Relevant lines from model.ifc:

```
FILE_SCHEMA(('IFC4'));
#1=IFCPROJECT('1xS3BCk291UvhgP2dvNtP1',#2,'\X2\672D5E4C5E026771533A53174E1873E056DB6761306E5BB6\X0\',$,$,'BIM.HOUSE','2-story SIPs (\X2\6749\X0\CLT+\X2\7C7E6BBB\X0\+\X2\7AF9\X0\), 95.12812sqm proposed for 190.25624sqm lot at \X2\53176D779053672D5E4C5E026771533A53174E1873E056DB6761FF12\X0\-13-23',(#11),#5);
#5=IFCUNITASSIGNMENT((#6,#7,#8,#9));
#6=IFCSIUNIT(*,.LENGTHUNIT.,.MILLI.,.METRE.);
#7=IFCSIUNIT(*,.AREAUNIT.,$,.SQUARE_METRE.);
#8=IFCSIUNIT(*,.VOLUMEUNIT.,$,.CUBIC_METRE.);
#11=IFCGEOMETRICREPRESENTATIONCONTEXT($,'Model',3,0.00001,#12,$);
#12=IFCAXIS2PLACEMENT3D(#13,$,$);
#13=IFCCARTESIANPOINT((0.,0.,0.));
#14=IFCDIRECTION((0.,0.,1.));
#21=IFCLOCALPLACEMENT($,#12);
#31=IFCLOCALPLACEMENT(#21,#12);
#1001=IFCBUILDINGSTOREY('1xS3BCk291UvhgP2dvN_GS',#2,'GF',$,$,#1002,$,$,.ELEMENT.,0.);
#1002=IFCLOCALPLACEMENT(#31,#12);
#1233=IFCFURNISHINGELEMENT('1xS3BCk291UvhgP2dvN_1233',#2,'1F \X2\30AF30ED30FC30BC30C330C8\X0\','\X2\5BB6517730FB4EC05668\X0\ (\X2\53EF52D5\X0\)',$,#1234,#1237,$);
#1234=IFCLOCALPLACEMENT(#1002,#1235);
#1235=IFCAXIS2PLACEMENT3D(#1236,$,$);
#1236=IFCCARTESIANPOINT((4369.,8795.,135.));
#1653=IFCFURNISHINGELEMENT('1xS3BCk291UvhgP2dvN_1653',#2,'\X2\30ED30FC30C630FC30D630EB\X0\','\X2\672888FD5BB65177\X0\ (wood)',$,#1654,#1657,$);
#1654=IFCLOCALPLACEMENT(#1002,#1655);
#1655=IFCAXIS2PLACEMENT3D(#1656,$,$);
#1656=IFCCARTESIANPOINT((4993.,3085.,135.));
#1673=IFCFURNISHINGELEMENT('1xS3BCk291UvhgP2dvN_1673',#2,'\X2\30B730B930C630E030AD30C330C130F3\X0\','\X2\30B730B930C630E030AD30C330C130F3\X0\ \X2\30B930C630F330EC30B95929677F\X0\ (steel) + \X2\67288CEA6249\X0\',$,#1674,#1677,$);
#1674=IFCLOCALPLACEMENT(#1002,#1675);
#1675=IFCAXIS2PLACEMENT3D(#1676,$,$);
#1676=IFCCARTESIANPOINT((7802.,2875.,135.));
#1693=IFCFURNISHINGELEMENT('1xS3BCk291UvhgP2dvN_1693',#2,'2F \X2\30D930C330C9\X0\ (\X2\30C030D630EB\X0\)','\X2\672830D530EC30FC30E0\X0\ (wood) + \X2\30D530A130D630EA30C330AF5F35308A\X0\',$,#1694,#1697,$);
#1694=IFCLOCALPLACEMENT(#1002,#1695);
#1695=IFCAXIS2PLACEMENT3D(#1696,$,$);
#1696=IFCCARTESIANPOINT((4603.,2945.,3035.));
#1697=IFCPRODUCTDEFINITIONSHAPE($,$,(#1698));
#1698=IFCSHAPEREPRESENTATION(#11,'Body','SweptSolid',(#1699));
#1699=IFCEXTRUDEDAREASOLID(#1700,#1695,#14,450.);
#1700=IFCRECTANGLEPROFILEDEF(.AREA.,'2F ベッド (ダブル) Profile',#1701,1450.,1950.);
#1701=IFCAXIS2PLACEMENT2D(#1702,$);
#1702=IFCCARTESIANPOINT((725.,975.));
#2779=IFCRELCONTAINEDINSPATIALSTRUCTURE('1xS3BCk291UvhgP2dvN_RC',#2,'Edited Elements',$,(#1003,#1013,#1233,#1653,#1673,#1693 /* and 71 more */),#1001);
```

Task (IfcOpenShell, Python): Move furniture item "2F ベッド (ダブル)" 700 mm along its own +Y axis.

```python
import ifcopenshell
import ifcopenshell.api.geometry
import ifcopenshell.util.placement
import ifcopenshell.util.unit

model = ifcopenshell.open("model.ifc")
unit_scale = ifcopenshell.util.unit.calculate_unit_scale(model)

item = model.by_guid("1xS3BCk291UvhgP2dvN_1693")
matrix = ifcopenshell.util.placement.get_local_placement(item.ObjectPlacement)
matrix[:3, 3] += matrix[:3, 1] * 0.7 / unit_scale
ifcopenshell.api.geometry.edit_object_placement(model, product=item, matrix=matrix, is_si=False)

print(ifcopenshell.util.placement.get_local_placement(item.ObjectPlacement).round(3) + 0.0)

model.write("model_updated.ifc")
```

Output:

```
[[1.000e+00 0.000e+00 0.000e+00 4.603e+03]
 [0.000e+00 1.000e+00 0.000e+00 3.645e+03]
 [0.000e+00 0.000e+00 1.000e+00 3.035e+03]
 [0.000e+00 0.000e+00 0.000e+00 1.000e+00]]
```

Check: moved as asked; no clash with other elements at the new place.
